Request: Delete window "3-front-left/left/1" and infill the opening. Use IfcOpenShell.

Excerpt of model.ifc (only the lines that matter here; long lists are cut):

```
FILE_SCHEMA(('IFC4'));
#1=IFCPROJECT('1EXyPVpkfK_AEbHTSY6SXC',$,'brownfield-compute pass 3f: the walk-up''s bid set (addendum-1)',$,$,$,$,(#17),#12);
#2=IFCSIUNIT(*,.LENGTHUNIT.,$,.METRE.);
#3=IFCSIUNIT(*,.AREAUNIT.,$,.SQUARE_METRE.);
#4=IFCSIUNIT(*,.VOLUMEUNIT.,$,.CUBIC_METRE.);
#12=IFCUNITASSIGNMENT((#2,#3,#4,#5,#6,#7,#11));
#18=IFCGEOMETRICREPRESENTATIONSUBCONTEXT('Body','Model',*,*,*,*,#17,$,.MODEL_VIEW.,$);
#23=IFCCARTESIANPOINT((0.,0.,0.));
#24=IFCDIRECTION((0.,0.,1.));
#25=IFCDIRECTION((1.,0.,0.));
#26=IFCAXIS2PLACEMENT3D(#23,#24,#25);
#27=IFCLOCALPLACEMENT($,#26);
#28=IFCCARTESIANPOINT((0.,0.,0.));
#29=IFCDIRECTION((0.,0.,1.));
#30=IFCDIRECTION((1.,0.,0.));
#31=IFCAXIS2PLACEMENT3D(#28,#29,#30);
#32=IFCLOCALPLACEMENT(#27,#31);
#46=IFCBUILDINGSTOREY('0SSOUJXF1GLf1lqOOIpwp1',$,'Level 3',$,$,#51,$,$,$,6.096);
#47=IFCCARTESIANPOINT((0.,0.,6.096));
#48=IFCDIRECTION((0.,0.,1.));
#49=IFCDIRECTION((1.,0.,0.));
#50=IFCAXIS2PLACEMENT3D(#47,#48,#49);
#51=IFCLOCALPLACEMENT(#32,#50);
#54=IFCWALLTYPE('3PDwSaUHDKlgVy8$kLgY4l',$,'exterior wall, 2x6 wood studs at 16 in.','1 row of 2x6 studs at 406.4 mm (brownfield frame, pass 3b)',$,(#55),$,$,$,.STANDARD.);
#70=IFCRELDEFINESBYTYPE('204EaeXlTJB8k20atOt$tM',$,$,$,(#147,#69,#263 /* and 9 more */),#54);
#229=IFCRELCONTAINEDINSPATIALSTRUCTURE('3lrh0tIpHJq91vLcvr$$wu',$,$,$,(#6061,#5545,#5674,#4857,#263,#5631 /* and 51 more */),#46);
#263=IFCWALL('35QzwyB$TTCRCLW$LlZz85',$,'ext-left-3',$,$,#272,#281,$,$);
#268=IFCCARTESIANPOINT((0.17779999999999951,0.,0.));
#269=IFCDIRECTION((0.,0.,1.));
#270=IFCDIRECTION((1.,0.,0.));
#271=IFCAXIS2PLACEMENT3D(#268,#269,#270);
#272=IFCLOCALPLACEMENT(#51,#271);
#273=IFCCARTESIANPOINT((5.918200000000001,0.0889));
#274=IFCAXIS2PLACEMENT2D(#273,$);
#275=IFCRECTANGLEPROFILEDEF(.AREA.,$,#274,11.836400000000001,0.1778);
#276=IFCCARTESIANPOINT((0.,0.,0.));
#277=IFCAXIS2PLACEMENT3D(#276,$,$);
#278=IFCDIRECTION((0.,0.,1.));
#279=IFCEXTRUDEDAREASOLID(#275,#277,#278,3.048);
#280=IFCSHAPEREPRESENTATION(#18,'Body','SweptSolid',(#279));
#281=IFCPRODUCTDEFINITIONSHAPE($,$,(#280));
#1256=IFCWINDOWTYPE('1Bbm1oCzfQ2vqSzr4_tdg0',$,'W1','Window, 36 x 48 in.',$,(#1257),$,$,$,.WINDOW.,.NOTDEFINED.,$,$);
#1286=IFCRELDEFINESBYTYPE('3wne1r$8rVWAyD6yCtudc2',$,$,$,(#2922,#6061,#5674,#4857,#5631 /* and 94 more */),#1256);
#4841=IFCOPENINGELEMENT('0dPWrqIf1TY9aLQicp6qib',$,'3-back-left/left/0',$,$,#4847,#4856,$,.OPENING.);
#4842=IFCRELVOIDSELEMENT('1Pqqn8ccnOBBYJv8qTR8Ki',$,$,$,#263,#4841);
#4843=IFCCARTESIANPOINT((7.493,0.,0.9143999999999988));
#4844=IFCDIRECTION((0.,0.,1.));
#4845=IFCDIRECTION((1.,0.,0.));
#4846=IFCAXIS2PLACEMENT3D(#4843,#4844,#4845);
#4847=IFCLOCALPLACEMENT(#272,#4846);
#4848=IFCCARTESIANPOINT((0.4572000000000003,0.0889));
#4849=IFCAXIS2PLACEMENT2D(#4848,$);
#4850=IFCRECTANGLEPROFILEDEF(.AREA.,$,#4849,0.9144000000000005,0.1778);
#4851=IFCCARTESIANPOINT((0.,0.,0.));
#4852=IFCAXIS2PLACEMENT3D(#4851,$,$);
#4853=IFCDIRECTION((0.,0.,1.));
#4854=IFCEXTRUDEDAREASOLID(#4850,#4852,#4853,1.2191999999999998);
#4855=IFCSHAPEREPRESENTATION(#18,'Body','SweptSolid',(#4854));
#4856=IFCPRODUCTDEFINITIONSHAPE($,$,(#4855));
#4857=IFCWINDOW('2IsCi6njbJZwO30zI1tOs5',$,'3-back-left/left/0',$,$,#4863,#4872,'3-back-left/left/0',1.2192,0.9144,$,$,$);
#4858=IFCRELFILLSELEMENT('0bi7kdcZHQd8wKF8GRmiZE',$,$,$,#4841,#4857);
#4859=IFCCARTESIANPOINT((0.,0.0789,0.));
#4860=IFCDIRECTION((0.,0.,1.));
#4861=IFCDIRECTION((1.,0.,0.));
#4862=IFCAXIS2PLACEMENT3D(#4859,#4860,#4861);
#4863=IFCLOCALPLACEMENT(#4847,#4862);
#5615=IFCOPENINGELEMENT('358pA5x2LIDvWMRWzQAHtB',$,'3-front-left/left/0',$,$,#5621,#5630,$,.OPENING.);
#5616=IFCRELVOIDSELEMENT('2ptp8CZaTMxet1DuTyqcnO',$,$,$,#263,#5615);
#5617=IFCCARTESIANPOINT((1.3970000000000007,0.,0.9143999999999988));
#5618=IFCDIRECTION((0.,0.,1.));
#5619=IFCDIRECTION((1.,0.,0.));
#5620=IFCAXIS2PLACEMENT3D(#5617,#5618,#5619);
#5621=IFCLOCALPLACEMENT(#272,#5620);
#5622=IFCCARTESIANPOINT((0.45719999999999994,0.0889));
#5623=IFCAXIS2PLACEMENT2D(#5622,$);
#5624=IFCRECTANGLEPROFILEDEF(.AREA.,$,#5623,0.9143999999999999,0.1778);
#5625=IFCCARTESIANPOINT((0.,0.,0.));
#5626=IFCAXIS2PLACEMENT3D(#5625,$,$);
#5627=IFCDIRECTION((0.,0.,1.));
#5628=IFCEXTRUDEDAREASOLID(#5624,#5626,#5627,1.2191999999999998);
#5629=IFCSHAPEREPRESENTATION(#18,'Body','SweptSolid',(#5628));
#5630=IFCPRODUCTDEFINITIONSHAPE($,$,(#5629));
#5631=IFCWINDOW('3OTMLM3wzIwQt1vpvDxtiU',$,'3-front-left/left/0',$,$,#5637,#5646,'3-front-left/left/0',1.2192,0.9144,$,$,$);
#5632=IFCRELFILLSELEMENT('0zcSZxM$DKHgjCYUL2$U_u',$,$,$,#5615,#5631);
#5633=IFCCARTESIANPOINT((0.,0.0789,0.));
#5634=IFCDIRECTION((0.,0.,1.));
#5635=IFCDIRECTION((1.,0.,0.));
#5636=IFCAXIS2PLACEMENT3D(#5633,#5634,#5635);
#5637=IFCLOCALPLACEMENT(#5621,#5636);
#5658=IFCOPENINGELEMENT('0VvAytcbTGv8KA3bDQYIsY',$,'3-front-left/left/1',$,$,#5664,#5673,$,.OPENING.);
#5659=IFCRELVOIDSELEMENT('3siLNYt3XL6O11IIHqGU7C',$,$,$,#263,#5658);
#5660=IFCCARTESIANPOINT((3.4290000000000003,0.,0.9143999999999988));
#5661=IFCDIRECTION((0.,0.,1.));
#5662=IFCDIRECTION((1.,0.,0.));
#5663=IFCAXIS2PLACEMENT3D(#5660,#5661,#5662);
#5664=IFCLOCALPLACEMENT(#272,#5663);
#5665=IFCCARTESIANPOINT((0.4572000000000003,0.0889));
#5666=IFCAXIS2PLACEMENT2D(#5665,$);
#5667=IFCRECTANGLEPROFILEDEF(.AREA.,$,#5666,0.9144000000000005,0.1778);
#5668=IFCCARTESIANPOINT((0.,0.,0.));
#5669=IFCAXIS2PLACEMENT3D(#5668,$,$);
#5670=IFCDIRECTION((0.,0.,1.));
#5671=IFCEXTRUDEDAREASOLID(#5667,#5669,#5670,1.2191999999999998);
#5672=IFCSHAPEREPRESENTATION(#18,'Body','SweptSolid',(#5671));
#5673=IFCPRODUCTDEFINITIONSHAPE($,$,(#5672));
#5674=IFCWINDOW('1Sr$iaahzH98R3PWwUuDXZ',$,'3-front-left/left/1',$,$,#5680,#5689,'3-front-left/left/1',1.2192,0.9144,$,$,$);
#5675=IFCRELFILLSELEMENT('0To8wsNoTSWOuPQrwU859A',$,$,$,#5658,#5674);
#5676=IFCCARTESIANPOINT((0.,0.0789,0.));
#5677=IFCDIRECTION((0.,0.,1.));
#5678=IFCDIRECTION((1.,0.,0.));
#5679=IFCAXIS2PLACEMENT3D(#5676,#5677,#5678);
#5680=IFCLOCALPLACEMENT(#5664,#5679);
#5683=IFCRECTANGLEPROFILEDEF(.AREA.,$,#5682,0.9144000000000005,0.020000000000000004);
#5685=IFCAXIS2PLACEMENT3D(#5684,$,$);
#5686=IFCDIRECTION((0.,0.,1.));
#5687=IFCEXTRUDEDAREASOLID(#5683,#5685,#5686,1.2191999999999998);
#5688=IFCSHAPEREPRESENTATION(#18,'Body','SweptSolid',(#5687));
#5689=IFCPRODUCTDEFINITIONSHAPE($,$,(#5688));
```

```python
import ifcopenshell
import ifcopenshell.api.feature
import ifcopenshell.api.root
import ifcopenshell.geom
import ifcopenshell.util.shape

model = ifcopenshell.open("model.ifc")
settings = ifcopenshell.geom.settings()


def volume(element):
    """Net volume in cubic metres, openings subtracted."""
    shape = ifcopenshell.geom.create_shape(settings, element)
    return ifcopenshell.util.shape.get_volume(shape.geometry)


window = model.by_id(5674)
opening = window.FillsVoids[0].RelatingOpeningElement
wall = opening.VoidsElements[0].RelatingBuildingElement
before = volume(wall)

ifcopenshell.api.root.remove_product(model, product=window)
ifcopenshell.api.feature.remove_feature(model, feature=opening)

after = volume(wall)

print(f"wall volume {before:.3f} -> {after:.3f} m3")

model.write("model_updated.ifc")
```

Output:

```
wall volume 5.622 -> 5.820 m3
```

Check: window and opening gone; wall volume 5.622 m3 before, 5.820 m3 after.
